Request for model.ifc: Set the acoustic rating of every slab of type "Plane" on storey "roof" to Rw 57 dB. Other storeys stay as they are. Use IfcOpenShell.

First a look at what the model holds.

```python
import ifcopenshell
import ifcopenshell.util.element

model = ifcopenshell.open("model.ifc")
print(model.schema)
storey = next(s for s in model.by_type("IfcBuildingStorey") if s.Name == "roof")
slabs = [e for e in ifcopenshell.util.element.get_decomposition(storey) if e.is_a("IfcSlab")]
seen = {}
for e in slabs:
    element_type = ifcopenshell.util.element.get_type(e)
    key = (element_type.Name if element_type != e and element_type else None, ifcopenshell.util.element.get_pset(e, "Pset_SlabCommon", "AcousticRating"))
    seen[key] = seen.get(key, 0) + 1
for (name, value), count in sorted(seen.items(), key=str):
    print(count, "x", name, "|", value)
```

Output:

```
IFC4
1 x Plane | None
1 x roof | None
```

```python
import ifcopenshell
import ifcopenshell.api.pset
import ifcopenshell.util.element

model = ifcopenshell.open("model.ifc")

storey = next(s for s in model.by_type("IfcBuildingStorey") if s.Name == "roof")
slabs = [e for e in ifcopenshell.util.element.get_decomposition(storey) if e.is_a("IfcSlab")]

count = 0
for e in slabs:
    element_type = ifcopenshell.util.element.get_type(e)
    if element_type in (None, e) or element_type.Name != "Plane":
        continue
    # add_pset returns the element's existing set when there is one.
    pset = ifcopenshell.api.pset.add_pset(model, product=e, name="Pset_SlabCommon")
    ifcopenshell.api.pset.edit_pset(model, pset=pset, properties={"AcousticRating": "Rw 57 dB"})
    count += 1

print(count, "slabs updated")

model.write("model_rev.ifc")
```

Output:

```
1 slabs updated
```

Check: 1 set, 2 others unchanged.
